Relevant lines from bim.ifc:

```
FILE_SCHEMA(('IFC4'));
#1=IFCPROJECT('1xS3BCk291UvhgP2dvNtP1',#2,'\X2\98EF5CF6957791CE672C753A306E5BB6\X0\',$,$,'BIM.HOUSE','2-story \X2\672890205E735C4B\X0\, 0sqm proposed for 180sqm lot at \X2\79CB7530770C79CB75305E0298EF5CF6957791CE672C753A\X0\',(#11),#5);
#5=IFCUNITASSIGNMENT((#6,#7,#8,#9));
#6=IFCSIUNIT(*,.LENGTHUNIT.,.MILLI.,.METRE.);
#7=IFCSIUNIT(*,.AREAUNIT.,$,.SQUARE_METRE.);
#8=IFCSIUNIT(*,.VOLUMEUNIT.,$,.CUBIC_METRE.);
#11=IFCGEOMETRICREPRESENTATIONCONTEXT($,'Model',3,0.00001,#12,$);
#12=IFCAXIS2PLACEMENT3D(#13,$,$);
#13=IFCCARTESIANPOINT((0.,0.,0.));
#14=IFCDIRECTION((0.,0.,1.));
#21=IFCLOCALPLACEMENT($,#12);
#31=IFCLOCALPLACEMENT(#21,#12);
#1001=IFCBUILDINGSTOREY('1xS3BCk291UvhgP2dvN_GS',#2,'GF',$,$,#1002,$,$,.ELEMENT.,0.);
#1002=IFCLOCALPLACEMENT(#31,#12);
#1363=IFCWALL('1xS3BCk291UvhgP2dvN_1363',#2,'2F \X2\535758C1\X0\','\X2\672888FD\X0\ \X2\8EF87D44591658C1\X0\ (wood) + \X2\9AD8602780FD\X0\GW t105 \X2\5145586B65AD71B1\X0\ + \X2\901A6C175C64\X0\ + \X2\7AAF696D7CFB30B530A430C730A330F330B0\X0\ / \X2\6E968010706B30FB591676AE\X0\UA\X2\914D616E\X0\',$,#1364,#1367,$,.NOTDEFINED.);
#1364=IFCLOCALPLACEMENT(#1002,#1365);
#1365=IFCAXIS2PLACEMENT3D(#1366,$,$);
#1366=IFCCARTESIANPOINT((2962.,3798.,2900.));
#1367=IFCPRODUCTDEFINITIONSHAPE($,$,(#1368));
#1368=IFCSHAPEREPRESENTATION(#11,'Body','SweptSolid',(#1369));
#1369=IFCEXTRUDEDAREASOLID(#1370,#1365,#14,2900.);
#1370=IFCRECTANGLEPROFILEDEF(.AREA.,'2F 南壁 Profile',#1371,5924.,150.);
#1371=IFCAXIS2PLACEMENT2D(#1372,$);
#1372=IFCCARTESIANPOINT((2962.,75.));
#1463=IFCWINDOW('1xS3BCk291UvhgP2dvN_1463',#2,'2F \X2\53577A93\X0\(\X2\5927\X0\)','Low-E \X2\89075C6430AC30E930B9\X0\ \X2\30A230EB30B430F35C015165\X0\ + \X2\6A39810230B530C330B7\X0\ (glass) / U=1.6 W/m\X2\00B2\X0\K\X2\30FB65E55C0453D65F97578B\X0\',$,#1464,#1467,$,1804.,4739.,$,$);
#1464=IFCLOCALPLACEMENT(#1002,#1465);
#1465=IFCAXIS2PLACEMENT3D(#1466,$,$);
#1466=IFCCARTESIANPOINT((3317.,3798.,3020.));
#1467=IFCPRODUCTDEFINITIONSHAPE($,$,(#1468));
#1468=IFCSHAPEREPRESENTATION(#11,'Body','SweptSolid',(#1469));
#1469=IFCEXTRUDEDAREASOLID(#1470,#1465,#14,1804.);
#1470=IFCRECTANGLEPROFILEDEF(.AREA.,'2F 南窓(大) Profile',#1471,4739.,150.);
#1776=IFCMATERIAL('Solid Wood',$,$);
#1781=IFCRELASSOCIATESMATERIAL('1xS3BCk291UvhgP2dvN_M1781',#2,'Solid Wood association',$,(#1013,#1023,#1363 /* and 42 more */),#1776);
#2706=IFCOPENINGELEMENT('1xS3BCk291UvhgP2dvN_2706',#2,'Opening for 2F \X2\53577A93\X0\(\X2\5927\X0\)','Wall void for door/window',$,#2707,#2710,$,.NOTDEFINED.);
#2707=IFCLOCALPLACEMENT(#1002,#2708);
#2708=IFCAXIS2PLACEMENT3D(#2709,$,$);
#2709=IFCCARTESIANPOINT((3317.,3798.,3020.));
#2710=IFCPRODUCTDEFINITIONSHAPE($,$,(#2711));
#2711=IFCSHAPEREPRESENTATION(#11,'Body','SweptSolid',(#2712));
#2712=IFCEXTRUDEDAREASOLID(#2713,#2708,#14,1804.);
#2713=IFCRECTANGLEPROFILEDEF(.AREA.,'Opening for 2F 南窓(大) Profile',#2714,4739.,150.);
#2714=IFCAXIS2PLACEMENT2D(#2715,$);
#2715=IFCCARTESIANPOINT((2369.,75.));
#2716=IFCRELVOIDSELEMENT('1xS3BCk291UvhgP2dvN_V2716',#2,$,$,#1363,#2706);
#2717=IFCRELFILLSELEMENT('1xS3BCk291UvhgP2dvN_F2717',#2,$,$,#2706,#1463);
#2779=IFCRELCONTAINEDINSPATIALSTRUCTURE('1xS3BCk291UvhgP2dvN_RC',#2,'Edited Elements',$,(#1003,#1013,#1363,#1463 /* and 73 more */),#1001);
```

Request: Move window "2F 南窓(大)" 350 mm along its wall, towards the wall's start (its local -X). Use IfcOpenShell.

```python
import ifcopenshell
import ifcopenshell.api.geometry
import ifcopenshell.util.placement
import ifcopenshell.util.unit

model = ifcopenshell.open("bim.ifc")
unit_scale = ifcopenshell.util.unit.calculate_unit_scale(model)

window = model.by_id(1463)
opening = window.FillsVoids[0].RelatingOpeningElement
wall = opening.VoidsElements[0].RelatingBuildingElement

wall_matrix = ifcopenshell.util.placement.get_local_placement(wall.ObjectPlacement)
shift = wall_matrix[:3, 0] * -0.35 / unit_scale
before = ifcopenshell.util.placement.get_local_placement(window.ObjectPlacement)[:3, 3].copy()

# The window is not placed relative to its opening, so move both.
for product in (opening, window):
    matrix = ifcopenshell.util.placement.get_local_placement(product.ObjectPlacement)
    matrix[:3, 3] += shift
    ifcopenshell.api.geometry.edit_object_placement(model, product=product, matrix=matrix, is_si=False)

after = ifcopenshell.util.placement.get_local_placement(window.ObjectPlacement)[:3, 3]
print("window moved by", (after - before).round(3) + 0.0)

model.write("bim_updated.ifc")
```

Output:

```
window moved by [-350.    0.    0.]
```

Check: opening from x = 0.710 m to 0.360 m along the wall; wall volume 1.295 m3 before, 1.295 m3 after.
